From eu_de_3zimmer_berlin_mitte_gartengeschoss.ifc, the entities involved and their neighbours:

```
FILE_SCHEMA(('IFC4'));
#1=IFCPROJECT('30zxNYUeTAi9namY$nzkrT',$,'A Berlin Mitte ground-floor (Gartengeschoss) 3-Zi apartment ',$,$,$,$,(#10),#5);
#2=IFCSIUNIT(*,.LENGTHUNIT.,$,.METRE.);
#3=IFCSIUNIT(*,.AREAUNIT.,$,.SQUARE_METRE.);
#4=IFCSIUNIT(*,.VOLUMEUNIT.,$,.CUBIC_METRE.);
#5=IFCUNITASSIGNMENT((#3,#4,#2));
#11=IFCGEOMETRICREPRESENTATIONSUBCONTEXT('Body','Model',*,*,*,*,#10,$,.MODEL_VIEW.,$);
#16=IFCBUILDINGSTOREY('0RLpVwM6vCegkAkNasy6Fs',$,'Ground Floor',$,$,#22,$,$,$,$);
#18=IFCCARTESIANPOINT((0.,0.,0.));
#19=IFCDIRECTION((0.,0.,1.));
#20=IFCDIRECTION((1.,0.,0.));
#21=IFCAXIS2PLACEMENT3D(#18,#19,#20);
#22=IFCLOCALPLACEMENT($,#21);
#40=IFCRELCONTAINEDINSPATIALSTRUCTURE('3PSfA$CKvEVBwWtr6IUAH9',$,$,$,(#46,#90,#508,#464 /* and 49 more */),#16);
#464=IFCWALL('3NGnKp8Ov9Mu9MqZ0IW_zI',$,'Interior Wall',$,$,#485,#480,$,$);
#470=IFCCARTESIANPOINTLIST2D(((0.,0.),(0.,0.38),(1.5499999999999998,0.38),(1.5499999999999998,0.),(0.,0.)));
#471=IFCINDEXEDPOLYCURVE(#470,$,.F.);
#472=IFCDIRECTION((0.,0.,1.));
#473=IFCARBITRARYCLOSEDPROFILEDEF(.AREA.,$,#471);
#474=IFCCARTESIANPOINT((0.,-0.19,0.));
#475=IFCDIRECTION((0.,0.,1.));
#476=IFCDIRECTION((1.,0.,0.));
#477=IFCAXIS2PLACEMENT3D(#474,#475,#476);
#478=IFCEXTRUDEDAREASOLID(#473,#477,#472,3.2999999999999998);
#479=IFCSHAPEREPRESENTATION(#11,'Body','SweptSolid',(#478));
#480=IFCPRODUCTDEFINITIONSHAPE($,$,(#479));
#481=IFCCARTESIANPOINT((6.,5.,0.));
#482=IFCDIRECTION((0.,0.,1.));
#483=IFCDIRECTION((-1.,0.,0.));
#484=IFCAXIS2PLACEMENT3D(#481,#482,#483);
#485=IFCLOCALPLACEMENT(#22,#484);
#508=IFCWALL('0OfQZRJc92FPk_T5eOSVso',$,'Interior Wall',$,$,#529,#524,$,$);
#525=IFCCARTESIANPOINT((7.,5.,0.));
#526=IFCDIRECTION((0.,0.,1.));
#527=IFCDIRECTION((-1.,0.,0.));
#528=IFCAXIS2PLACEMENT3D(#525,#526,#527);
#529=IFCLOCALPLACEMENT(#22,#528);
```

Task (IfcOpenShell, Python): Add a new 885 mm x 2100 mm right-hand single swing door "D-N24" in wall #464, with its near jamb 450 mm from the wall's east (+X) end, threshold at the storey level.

```python
import numpy as np
import ifcopenshell
import ifcopenshell.api.feature
import ifcopenshell.api.geometry
import ifcopenshell.api.root
import ifcopenshell.api.spatial
import ifcopenshell.geom
import ifcopenshell.util.element
import ifcopenshell.util.placement
import ifcopenshell.util.representation
import ifcopenshell.util.shape
import ifcopenshell.util.unit

model = ifcopenshell.open("eu_de_3zimmer_berlin_mitte_gartengeschoss.ifc")
unit_scale = ifcopenshell.util.unit.calculate_unit_scale(model)
settings = ifcopenshell.geom.settings()


def volume(element):
    """Net volume in cubic metres, openings subtracted."""
    shape = ifcopenshell.geom.create_shape(settings, element)
    return ifcopenshell.util.shape.get_volume(shape.geometry)


wall = model.by_guid("3NGnKp8Ov9Mu9MqZ0IW_zI")
storey = ifcopenshell.util.element.get_container(wall, ifc_class="IfcBuildingStorey")
context = ifcopenshell.util.representation.get_context(model, "Model", "Body", "MODEL_VIEW")
before = volume(wall)

width, height, from_end, sill = 0.885, 2.1, 0.45, 0.0  # metres

# The wall runs along its own X axis, and the end named is its -X end.
wall_shape = ifcopenshell.geom.create_shape(settings, wall)
x, y, z = ifcopenshell.util.shape.get_vertices(wall_shape.geometry).T
start = x.min() + from_end
face, thickness = float(y.min()), float(y.max() - y.min())
wall_matrix = ifcopenshell.util.placement.get_local_placement(wall.ObjectPlacement)
level = ifcopenshell.util.placement.get_local_placement(storey.ObjectPlacement)[2, 3]


def in_wall(x, y):
    """Placement at x, y metres in the wall's axes, at sill height."""
    matrix = wall_matrix.copy()
    matrix[:, 3] = wall_matrix @ np.array([x / unit_scale, y / unit_scale, 0.0, 1.0])
    matrix[2, 3] = level + sill / unit_scale
    return matrix


# Opening: a box that overshoots both wall faces by 50 mm.
opening = ifcopenshell.api.root.create_entity(model, ifc_class="IfcOpeningElement", predefined_type="OPENING")
box = ifcopenshell.api.geometry.add_wall_representation(
    model, context=context, length=width, height=height, thickness=thickness + 0.1
)
ifcopenshell.api.geometry.assign_representation(model, product=opening, representation=box)
ifcopenshell.api.geometry.edit_object_placement(model, product=opening, matrix=in_wall(start, face - 0.05), is_si=False)
ifcopenshell.api.feature.add_feature(model, feature=opening, element=wall)

door = ifcopenshell.api.root.create_entity(model, ifc_class="IfcDoor", name="D-N24", predefined_type="DOOR")
door.OverallWidth, door.OverallHeight = width / unit_scale, height / unit_scale
door.OperationType = "SINGLE_SWING_RIGHT"
body = ifcopenshell.api.geometry.add_door_representation(
    model,
    context=context,
    overall_width=door.OverallWidth,
    overall_height=door.OverallHeight,
    operation_type="SINGLE_SWING_RIGHT",
    lining_properties={"LiningDepth": thickness / unit_scale, "ThresholdDepth": thickness / unit_scale},
)
ifcopenshell.api.geometry.assign_representation(model, product=door, representation=body)
ifcopenshell.api.spatial.assign_container(model, products=[door], relating_structure=storey)
ifcopenshell.api.feature.add_filling(model, opening=opening, element=door)

# The lining spans the wall, so the door starts at the wall face.
ifcopenshell.api.geometry.edit_object_placement(model, product=door, matrix=in_wall(start, face), is_si=False)

after = volume(wall)

print(f"wall volume {before:.3f} -> {after:.3f} m3")

model.write("eu_de_3zimmer_berlin_mitte_gartengeschoss_updated.ifc")
```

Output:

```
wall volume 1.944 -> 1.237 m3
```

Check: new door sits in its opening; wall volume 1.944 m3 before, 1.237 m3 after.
